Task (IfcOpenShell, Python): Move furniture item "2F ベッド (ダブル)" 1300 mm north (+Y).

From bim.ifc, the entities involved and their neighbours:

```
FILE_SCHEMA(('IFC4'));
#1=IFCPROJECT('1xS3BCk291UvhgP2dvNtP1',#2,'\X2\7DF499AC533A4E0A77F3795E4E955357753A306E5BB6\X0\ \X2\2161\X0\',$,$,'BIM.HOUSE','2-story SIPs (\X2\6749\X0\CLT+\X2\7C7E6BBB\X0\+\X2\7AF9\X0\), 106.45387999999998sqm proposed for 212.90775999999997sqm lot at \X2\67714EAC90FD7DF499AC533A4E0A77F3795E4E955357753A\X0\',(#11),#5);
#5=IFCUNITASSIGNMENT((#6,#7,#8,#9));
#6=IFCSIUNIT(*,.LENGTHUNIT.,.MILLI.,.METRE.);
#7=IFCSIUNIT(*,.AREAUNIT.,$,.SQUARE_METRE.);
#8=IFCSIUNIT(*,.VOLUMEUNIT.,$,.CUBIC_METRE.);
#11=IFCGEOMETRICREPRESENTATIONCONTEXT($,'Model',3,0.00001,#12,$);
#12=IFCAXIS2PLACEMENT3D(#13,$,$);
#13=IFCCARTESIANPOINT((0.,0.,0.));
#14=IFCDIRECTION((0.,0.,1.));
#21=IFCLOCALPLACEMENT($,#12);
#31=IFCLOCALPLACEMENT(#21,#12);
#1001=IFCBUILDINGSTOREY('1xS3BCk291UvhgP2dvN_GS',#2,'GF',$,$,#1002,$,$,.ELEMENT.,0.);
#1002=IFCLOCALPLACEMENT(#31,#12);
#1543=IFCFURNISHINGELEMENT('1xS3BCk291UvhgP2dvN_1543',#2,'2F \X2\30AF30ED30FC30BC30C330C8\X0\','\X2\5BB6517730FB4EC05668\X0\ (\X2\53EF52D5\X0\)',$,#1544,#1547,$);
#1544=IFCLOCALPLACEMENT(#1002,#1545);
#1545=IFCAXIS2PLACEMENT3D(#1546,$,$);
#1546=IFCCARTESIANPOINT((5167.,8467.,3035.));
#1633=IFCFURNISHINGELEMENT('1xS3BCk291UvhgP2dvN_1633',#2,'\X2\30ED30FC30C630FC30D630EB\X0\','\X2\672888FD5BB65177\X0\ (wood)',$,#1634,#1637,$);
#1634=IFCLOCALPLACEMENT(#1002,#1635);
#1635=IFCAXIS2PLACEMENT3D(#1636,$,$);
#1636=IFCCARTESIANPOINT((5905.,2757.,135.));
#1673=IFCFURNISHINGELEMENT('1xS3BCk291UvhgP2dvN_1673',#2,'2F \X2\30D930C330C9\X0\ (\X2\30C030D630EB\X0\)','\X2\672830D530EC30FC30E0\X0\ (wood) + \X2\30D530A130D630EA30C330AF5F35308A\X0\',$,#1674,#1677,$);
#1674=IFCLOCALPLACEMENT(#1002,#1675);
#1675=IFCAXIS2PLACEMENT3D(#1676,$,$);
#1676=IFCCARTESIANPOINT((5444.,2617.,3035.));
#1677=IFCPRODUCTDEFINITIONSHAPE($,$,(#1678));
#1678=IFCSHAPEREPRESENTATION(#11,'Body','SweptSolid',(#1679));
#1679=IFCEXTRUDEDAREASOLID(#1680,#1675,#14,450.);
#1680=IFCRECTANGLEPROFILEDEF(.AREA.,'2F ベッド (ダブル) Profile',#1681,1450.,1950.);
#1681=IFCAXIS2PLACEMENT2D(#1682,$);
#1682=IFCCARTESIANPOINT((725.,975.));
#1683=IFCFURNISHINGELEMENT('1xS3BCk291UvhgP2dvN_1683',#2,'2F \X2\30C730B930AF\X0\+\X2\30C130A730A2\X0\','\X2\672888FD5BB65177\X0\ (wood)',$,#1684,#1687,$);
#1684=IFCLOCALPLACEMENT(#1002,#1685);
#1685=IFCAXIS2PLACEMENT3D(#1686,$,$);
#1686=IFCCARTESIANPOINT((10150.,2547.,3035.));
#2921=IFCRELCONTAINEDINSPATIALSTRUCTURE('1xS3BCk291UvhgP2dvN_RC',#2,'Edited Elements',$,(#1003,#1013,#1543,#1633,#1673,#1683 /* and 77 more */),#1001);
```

```python
import ifcopenshell
import ifcopenshell.api.geometry
import ifcopenshell.util.placement

model = ifcopenshell.open("bim.ifc")

item = model.by_guid("1xS3BCk291UvhgP2dvN_1673")
matrix = ifcopenshell.util.placement.get_local_placement(item.ObjectPlacement)
matrix[1, 3] += 1300.0
ifcopenshell.api.geometry.edit_object_placement(model, product=item, matrix=matrix, is_si=False)

print(ifcopenshell.util.placement.get_local_placement(item.ObjectPlacement).round(3) + 0.0)

model.write("bim-out.ifc")
```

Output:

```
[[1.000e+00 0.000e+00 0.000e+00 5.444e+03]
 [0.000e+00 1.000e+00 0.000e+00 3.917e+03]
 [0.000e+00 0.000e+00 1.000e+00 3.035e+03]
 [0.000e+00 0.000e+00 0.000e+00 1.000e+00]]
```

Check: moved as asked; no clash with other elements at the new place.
